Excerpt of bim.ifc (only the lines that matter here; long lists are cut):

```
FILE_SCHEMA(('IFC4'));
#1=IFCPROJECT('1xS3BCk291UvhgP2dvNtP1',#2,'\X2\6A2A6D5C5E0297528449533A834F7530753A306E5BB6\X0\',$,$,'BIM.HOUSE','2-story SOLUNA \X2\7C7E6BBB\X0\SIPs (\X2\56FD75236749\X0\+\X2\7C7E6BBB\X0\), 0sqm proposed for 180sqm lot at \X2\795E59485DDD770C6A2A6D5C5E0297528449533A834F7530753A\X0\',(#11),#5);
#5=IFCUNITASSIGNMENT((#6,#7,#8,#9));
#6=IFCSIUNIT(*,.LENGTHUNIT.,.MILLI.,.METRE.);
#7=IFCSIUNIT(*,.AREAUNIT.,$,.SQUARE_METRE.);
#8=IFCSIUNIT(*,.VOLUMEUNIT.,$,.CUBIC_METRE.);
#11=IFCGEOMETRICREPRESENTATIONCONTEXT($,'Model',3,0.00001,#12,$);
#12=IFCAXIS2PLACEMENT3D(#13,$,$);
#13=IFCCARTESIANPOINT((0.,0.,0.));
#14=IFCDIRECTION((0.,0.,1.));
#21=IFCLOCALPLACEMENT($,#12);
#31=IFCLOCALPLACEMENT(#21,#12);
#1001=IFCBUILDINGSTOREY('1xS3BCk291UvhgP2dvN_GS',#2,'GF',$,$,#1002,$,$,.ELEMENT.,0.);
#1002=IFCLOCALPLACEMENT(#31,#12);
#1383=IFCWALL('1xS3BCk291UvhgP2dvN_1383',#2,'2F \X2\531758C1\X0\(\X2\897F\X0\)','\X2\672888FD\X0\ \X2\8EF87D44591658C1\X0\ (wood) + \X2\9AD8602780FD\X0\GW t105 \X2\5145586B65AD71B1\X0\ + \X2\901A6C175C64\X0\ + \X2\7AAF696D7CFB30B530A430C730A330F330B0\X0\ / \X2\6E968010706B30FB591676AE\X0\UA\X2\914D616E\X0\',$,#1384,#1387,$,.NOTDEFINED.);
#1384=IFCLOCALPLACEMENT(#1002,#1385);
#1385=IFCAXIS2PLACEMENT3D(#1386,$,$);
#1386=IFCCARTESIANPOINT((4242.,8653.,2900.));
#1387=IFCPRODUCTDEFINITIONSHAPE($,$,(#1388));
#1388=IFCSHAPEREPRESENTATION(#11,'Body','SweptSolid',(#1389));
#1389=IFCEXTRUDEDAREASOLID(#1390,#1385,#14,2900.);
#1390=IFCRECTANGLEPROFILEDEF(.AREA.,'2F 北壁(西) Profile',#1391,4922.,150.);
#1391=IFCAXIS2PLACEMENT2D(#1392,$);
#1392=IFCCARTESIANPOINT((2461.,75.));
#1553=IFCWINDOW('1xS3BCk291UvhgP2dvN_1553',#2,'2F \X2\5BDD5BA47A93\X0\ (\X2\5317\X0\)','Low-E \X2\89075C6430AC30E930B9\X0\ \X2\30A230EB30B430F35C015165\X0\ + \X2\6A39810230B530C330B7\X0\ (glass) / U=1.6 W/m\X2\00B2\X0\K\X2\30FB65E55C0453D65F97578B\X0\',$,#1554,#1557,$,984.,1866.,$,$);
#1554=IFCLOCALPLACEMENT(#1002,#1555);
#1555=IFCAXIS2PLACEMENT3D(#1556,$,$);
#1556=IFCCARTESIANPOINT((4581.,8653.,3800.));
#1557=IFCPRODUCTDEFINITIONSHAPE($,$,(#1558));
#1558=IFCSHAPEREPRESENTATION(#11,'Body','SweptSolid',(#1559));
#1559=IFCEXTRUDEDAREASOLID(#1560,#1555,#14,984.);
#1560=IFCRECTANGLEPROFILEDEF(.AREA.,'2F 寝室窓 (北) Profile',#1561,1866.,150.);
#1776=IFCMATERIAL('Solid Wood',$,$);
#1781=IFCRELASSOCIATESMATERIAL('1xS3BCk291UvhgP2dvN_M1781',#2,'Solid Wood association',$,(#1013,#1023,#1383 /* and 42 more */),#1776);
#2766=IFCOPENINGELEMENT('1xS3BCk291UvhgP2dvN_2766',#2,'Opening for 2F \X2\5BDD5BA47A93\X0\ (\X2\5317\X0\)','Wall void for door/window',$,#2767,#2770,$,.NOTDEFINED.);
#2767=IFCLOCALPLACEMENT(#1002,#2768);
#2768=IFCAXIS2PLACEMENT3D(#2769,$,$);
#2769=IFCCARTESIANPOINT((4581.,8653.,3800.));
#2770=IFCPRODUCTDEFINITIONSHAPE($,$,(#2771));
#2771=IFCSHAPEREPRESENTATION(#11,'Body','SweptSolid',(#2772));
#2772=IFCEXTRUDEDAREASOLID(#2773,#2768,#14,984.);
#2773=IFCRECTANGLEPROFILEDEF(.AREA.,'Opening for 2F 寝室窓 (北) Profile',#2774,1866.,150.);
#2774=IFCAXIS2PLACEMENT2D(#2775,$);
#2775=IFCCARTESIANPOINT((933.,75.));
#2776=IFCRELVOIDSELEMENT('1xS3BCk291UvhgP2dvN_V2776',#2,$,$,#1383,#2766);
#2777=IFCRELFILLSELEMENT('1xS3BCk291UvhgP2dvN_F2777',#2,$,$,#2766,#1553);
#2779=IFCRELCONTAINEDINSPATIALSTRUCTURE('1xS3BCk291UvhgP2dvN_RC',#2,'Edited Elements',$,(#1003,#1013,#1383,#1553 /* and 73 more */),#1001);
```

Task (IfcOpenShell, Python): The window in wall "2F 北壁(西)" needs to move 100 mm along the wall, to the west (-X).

```python
import ifcopenshell
import ifcopenshell.api.geometry
import ifcopenshell.util.placement

model = ifcopenshell.open("bim.ifc")

window = model.by_guid("1xS3BCk291UvhgP2dvN_1553")
opening = window.FillsVoids[0].RelatingOpeningElement
wall = opening.VoidsElements[0].RelatingBuildingElement

wall_matrix = ifcopenshell.util.placement.get_local_placement(wall.ObjectPlacement)
shift = wall_matrix[:3, 0] * -100.0
before = ifcopenshell.util.placement.get_local_placement(window.ObjectPlacement)[:3, 3].copy()

# The window is not placed relative to its opening, so move both.
for product in (opening, window):
    matrix = ifcopenshell.util.placement.get_local_placement(product.ObjectPlacement)
    matrix[:3, 3] += shift
    ifcopenshell.api.geometry.edit_object_placement(model, product=product, matrix=matrix, is_si=False)

after = ifcopenshell.util.placement.get_local_placement(window.ObjectPlacement)[:3, 3]
print("window moved by", (after - before).round(3) + 0.0)

model.write("bim_edited.ifc")
```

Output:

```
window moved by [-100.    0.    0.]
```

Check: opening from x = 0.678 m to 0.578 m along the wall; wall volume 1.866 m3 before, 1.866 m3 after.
